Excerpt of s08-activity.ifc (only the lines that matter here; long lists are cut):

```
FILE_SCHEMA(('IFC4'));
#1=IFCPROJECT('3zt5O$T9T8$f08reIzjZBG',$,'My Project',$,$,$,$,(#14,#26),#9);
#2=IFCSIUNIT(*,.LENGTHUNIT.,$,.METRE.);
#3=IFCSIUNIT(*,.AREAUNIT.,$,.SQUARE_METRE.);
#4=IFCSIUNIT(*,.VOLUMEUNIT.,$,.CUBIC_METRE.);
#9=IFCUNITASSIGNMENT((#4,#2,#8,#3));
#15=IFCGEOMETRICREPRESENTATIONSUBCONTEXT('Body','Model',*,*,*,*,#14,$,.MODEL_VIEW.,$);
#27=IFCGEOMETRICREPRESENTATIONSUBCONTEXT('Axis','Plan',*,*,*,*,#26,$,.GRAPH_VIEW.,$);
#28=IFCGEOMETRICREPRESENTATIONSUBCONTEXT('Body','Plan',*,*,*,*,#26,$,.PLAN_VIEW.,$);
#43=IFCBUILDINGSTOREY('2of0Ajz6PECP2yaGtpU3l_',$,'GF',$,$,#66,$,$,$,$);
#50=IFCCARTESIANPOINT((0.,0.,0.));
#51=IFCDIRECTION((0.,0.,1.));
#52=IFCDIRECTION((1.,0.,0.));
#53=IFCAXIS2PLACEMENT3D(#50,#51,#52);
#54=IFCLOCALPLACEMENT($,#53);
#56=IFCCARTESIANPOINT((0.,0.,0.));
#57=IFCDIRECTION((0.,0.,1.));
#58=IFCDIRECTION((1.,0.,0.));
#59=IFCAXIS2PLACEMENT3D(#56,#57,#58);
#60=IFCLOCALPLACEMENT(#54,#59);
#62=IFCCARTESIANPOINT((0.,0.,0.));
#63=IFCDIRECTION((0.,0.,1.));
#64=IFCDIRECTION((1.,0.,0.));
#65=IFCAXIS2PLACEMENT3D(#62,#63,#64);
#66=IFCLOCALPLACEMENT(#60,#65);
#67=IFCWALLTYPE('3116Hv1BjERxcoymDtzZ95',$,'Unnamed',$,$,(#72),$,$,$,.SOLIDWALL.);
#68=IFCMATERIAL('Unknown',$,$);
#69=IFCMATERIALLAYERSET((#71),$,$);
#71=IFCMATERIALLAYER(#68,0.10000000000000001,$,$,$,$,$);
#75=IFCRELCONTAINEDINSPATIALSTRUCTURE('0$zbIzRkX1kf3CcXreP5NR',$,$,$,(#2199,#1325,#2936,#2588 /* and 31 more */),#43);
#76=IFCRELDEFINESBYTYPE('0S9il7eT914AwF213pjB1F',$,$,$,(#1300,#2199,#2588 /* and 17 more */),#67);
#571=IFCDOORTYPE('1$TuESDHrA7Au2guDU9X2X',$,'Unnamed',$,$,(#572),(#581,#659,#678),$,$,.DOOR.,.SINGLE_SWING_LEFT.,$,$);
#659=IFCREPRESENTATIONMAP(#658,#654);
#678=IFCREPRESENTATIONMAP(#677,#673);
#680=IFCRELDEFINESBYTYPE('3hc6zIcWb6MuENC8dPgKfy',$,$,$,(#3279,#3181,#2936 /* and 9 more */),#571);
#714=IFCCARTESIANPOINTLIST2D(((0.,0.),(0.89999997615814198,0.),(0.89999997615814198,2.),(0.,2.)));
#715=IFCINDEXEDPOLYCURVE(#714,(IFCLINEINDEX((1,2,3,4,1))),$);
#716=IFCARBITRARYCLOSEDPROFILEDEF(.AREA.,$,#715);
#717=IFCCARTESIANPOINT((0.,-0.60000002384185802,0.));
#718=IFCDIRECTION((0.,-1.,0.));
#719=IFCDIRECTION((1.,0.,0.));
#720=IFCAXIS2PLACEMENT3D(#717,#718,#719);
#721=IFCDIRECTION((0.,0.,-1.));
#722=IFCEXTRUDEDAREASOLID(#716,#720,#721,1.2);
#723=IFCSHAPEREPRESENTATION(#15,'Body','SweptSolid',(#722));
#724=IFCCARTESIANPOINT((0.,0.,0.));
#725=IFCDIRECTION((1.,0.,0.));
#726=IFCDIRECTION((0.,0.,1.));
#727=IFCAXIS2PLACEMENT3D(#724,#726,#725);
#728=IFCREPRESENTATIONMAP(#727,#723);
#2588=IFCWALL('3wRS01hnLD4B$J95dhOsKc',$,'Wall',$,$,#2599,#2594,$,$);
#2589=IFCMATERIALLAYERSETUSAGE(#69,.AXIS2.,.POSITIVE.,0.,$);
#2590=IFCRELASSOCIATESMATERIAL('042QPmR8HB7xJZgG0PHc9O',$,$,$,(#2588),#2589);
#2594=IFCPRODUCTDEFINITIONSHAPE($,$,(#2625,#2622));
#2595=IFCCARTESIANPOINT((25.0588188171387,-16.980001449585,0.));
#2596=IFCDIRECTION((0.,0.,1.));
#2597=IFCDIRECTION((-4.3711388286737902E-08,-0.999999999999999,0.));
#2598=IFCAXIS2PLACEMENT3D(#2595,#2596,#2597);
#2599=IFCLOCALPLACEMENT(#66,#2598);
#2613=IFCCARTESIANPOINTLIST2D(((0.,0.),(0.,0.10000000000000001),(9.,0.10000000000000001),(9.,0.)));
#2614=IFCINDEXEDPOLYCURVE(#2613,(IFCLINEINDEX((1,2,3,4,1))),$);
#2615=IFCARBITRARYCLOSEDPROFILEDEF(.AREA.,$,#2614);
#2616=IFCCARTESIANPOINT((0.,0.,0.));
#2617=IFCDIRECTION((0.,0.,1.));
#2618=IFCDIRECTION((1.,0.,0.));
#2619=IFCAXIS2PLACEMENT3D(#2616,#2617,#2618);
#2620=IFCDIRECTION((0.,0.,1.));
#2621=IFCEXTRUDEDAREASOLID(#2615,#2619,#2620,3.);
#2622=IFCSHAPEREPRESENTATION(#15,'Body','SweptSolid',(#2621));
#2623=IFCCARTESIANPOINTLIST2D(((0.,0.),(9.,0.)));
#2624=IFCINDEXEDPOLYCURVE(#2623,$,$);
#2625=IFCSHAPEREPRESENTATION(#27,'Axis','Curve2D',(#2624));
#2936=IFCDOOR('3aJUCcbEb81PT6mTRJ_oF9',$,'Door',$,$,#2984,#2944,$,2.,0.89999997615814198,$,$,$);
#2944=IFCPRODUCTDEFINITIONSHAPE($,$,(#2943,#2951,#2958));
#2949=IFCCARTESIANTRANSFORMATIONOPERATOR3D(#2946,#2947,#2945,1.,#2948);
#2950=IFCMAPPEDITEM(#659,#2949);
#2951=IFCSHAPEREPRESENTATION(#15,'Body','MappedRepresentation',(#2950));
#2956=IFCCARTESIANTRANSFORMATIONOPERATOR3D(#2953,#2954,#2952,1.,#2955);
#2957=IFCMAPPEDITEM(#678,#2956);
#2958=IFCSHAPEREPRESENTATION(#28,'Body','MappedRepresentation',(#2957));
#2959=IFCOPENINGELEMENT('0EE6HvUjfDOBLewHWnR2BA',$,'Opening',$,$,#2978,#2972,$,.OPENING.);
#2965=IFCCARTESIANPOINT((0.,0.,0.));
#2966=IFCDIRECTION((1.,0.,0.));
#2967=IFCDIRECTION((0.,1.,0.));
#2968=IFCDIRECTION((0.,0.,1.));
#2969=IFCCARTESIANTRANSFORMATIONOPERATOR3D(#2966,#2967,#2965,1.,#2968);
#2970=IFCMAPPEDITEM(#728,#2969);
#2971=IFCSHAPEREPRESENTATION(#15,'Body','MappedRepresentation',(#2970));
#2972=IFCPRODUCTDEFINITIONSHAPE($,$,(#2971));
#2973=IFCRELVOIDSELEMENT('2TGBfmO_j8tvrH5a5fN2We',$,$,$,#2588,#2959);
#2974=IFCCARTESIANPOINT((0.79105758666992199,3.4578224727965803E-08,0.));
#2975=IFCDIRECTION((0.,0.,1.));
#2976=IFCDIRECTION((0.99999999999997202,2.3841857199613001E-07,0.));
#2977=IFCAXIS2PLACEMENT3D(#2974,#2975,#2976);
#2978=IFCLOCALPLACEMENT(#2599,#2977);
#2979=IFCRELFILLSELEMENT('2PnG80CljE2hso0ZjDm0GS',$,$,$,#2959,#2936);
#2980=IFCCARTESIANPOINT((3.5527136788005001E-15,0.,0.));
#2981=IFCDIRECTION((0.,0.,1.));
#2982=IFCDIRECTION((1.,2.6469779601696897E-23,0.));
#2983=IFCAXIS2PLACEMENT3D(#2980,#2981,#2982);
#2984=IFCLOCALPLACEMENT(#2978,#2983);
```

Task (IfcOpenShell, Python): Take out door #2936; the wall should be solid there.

```python
import ifcopenshell
import ifcopenshell.api.feature
import ifcopenshell.api.root
import ifcopenshell.geom
import ifcopenshell.util.shape

model = ifcopenshell.open("s08-activity.ifc")
settings = ifcopenshell.geom.settings()


def volume(element):
    """Net volume in cubic metres, openings subtracted."""
    shape = ifcopenshell.geom.create_shape(settings, element)
    return ifcopenshell.util.shape.get_volume(shape.geometry)


door = model.by_guid("3aJUCcbEb81PT6mTRJ_oF9")
opening = door.FillsVoids[0].RelatingOpeningElement
wall = opening.VoidsElements[0].RelatingBuildingElement
before = volume(wall)

ifcopenshell.api.root.remove_product(model, product=door)
ifcopenshell.api.feature.remove_feature(model, feature=opening)

after = volume(wall)

print(f"wall volume {before:.3f} -> {after:.3f} m3")

model.write("s08-activity_v2.ifc")
```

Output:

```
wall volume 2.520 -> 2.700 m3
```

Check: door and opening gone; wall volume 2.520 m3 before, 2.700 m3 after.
